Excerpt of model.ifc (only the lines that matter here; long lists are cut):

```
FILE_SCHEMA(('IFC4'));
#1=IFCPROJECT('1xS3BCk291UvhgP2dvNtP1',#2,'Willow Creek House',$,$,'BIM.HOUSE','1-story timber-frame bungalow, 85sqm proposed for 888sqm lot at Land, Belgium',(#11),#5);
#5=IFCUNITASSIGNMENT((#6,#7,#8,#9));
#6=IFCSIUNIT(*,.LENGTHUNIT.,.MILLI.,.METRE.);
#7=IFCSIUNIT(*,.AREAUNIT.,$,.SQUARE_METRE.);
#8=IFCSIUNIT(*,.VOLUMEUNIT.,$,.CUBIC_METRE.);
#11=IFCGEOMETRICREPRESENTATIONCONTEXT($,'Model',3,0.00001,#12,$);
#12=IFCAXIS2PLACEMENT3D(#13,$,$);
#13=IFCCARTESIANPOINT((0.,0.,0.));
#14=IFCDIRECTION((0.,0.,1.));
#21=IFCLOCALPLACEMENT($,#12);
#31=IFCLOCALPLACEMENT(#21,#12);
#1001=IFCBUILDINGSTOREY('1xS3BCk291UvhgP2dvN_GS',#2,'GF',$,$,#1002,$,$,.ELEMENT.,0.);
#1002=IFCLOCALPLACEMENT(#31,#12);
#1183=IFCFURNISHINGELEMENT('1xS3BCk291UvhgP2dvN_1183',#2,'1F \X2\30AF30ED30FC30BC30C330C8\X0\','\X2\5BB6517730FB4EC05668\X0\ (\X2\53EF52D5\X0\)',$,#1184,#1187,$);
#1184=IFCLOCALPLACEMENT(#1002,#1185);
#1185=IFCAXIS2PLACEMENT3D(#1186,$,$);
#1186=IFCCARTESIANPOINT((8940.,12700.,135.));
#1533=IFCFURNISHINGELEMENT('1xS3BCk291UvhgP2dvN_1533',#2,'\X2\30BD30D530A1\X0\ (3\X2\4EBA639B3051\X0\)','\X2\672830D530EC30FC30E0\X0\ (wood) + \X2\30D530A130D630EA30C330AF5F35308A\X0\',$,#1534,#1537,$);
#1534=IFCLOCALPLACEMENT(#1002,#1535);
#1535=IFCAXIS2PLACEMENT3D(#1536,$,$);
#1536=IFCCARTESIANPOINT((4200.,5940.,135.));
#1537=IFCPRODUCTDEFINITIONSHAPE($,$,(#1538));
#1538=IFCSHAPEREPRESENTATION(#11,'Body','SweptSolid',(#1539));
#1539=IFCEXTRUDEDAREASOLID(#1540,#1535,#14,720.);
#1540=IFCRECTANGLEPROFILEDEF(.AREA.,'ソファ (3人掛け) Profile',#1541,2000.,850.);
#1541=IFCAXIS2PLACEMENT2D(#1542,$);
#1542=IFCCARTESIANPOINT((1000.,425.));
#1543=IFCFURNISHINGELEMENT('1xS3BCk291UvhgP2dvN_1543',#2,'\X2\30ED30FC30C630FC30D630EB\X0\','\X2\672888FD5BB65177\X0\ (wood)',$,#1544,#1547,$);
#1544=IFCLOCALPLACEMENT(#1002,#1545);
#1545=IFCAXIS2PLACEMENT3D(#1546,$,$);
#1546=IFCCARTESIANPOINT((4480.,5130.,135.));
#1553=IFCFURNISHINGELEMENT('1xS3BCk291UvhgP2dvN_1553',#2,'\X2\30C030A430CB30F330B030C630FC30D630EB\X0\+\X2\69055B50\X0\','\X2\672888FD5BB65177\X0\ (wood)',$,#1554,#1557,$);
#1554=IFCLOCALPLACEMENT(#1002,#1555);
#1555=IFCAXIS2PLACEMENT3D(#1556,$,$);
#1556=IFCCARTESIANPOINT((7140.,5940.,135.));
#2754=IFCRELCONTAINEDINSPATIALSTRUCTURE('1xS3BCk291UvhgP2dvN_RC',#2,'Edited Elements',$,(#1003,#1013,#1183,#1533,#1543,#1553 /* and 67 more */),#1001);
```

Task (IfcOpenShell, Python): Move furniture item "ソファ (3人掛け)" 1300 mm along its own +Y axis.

```python
import ifcopenshell
import ifcopenshell.api.geometry
import ifcopenshell.util.placement
import ifcopenshell.util.unit

model = ifcopenshell.open("model.ifc")
unit_scale = ifcopenshell.util.unit.calculate_unit_scale(model)

item = model.by_id(1533)
matrix = ifcopenshell.util.placement.get_local_placement(item.ObjectPlacement)
matrix[:3, 3] += matrix[:3, 1] * 1.3 / unit_scale
ifcopenshell.api.geometry.edit_object_placement(model, product=item, matrix=matrix, is_si=False)

print(ifcopenshell.util.placement.get_local_placement(item.ObjectPlacement).round(3) + 0.0)

model.write("model_updated.ifc")
```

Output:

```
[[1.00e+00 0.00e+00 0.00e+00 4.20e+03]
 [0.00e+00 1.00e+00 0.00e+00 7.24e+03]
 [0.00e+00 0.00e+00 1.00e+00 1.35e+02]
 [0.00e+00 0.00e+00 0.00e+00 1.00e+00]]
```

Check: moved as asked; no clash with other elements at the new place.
